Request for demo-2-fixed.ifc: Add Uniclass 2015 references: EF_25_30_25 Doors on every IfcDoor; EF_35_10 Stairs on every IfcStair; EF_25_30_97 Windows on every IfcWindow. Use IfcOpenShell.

First a look at what the model holds.

```python
import ifcopenshell

model = ifcopenshell.open("demo-2-fixed.ifc")
print(model.schema)
print("classifications:", [c.Name for c in model.by_type("IfcClassification")])
for ifc_class in ("IfcDoor", "IfcRoof", "IfcStair", "IfcWall", "IfcWindow"):
    print(ifc_class, len(model.by_type(ifc_class)))
```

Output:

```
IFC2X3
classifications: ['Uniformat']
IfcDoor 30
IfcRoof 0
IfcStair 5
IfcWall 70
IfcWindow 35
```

```python
import ifcopenshell
import ifcopenshell.api.classification

model = ifcopenshell.open("demo-2-fixed.ifc")

# IFC2X3 requires Source and Edition and has no link from the project to the system.
system = model.create_entity("IfcClassification", Source="NBS", Edition="2015", Name="Uniclass 2015")

codes = {
    "IfcDoor": ("EF_25_30_25", "Doors"),
    "IfcStair": ("EF_35_10", "Stairs"),
    "IfcWindow": ("EF_25_30_97", "Windows"),
}
for ifc_class, (code, name) in codes.items():
    products = model.by_type(ifc_class)
    ifcopenshell.api.classification.add_reference(
        model, products=products, classification=system, identification=code, name=name
    )
    print(code, len(products))

model.write("demo-2-fixed_updated.ifc")
```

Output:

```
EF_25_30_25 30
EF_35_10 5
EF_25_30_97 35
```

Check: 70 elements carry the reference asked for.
